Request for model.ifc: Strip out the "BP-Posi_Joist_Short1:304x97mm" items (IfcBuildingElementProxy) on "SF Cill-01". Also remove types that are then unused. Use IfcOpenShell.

First a look at what the model holds.

```python
import ifcopenshell
import ifcopenshell.util.element

model = ifcopenshell.open("model.ifc")
print(model.schema)
storey = next(s for s in model.by_type("IfcBuildingStorey") if s.Name == "SF Cill-01")
proxies = [e for e in ifcopenshell.util.element.get_decomposition(storey) if e.is_a("IfcBuildingElementProxy")]
seen = {}
for e in proxies:
    element_type = ifcopenshell.util.element.get_type(e)
    name = element_type.Name if element_type not in (None, e) else None
    seen[name] = seen.get(name, 0) + 1
for name, count in sorted(seen.items(), key=str):
    print(count, "x", name)
```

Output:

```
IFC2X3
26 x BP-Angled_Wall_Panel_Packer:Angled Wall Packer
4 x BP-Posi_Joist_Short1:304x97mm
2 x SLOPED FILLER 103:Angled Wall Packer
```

```python
import ifcopenshell
import ifcopenshell.api.root
import ifcopenshell.util.element

model = ifcopenshell.open("model.ifc")

storey = next(s for s in model.by_type("IfcBuildingStorey") if s.Name == "SF Cill-01")
proxies = [e for e in ifcopenshell.util.element.get_decomposition(storey) if e.is_a("IfcBuildingElementProxy")]
targets = [e for e in proxies if (t := ifcopenshell.util.element.get_type(e)) not in (None, e) and t.Name == "BP-Posi_Joist_Short1:304x97mm"]
types = {ifcopenshell.util.element.get_type(e) for e in targets} - {None, *targets}

for e in targets:
    ifcopenshell.api.root.remove_product(model, product=e)
print(len(targets), "removed")

unused = [t for t in types if not ifcopenshell.util.element.get_types(t)]
for t in unused:
    ifcopenshell.api.root.remove_product(model, product=t)
print(len(unused), "unused types removed")

model.write("model-out.ifc")
```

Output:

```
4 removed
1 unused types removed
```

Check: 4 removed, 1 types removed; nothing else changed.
